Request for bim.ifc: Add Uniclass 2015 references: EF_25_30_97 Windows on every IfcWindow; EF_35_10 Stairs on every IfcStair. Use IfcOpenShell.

First a look at what the model holds.

```python
import ifcopenshell

model = ifcopenshell.open("bim.ifc")
print(model.schema)
print("classifications:", [c.Name for c in model.by_type("IfcClassification")])
for ifc_class in ("IfcDoor", "IfcRoof", "IfcStair", "IfcWall", "IfcWindow"):
    print(ifc_class, len(model.by_type(ifc_class)))
```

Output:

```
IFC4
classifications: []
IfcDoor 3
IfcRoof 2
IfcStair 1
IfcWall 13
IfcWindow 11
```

```python
import ifcopenshell
import ifcopenshell.api.classification

model = ifcopenshell.open("bim.ifc")

system = ifcopenshell.api.classification.add_classification(model, classification="Uniclass 2015")

codes = {
    "IfcWindow": ("EF_25_30_97", "Windows"),
    "IfcStair": ("EF_35_10", "Stairs"),
}
for ifc_class, (code, name) in codes.items():
    products = model.by_type(ifc_class)
    ifcopenshell.api.classification.add_reference(
        model, products=products, classification=system, identification=code, name=name
    )
    print(code, len(products))

model.write("bim_rev.ifc")
```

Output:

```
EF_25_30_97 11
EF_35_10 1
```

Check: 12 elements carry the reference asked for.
